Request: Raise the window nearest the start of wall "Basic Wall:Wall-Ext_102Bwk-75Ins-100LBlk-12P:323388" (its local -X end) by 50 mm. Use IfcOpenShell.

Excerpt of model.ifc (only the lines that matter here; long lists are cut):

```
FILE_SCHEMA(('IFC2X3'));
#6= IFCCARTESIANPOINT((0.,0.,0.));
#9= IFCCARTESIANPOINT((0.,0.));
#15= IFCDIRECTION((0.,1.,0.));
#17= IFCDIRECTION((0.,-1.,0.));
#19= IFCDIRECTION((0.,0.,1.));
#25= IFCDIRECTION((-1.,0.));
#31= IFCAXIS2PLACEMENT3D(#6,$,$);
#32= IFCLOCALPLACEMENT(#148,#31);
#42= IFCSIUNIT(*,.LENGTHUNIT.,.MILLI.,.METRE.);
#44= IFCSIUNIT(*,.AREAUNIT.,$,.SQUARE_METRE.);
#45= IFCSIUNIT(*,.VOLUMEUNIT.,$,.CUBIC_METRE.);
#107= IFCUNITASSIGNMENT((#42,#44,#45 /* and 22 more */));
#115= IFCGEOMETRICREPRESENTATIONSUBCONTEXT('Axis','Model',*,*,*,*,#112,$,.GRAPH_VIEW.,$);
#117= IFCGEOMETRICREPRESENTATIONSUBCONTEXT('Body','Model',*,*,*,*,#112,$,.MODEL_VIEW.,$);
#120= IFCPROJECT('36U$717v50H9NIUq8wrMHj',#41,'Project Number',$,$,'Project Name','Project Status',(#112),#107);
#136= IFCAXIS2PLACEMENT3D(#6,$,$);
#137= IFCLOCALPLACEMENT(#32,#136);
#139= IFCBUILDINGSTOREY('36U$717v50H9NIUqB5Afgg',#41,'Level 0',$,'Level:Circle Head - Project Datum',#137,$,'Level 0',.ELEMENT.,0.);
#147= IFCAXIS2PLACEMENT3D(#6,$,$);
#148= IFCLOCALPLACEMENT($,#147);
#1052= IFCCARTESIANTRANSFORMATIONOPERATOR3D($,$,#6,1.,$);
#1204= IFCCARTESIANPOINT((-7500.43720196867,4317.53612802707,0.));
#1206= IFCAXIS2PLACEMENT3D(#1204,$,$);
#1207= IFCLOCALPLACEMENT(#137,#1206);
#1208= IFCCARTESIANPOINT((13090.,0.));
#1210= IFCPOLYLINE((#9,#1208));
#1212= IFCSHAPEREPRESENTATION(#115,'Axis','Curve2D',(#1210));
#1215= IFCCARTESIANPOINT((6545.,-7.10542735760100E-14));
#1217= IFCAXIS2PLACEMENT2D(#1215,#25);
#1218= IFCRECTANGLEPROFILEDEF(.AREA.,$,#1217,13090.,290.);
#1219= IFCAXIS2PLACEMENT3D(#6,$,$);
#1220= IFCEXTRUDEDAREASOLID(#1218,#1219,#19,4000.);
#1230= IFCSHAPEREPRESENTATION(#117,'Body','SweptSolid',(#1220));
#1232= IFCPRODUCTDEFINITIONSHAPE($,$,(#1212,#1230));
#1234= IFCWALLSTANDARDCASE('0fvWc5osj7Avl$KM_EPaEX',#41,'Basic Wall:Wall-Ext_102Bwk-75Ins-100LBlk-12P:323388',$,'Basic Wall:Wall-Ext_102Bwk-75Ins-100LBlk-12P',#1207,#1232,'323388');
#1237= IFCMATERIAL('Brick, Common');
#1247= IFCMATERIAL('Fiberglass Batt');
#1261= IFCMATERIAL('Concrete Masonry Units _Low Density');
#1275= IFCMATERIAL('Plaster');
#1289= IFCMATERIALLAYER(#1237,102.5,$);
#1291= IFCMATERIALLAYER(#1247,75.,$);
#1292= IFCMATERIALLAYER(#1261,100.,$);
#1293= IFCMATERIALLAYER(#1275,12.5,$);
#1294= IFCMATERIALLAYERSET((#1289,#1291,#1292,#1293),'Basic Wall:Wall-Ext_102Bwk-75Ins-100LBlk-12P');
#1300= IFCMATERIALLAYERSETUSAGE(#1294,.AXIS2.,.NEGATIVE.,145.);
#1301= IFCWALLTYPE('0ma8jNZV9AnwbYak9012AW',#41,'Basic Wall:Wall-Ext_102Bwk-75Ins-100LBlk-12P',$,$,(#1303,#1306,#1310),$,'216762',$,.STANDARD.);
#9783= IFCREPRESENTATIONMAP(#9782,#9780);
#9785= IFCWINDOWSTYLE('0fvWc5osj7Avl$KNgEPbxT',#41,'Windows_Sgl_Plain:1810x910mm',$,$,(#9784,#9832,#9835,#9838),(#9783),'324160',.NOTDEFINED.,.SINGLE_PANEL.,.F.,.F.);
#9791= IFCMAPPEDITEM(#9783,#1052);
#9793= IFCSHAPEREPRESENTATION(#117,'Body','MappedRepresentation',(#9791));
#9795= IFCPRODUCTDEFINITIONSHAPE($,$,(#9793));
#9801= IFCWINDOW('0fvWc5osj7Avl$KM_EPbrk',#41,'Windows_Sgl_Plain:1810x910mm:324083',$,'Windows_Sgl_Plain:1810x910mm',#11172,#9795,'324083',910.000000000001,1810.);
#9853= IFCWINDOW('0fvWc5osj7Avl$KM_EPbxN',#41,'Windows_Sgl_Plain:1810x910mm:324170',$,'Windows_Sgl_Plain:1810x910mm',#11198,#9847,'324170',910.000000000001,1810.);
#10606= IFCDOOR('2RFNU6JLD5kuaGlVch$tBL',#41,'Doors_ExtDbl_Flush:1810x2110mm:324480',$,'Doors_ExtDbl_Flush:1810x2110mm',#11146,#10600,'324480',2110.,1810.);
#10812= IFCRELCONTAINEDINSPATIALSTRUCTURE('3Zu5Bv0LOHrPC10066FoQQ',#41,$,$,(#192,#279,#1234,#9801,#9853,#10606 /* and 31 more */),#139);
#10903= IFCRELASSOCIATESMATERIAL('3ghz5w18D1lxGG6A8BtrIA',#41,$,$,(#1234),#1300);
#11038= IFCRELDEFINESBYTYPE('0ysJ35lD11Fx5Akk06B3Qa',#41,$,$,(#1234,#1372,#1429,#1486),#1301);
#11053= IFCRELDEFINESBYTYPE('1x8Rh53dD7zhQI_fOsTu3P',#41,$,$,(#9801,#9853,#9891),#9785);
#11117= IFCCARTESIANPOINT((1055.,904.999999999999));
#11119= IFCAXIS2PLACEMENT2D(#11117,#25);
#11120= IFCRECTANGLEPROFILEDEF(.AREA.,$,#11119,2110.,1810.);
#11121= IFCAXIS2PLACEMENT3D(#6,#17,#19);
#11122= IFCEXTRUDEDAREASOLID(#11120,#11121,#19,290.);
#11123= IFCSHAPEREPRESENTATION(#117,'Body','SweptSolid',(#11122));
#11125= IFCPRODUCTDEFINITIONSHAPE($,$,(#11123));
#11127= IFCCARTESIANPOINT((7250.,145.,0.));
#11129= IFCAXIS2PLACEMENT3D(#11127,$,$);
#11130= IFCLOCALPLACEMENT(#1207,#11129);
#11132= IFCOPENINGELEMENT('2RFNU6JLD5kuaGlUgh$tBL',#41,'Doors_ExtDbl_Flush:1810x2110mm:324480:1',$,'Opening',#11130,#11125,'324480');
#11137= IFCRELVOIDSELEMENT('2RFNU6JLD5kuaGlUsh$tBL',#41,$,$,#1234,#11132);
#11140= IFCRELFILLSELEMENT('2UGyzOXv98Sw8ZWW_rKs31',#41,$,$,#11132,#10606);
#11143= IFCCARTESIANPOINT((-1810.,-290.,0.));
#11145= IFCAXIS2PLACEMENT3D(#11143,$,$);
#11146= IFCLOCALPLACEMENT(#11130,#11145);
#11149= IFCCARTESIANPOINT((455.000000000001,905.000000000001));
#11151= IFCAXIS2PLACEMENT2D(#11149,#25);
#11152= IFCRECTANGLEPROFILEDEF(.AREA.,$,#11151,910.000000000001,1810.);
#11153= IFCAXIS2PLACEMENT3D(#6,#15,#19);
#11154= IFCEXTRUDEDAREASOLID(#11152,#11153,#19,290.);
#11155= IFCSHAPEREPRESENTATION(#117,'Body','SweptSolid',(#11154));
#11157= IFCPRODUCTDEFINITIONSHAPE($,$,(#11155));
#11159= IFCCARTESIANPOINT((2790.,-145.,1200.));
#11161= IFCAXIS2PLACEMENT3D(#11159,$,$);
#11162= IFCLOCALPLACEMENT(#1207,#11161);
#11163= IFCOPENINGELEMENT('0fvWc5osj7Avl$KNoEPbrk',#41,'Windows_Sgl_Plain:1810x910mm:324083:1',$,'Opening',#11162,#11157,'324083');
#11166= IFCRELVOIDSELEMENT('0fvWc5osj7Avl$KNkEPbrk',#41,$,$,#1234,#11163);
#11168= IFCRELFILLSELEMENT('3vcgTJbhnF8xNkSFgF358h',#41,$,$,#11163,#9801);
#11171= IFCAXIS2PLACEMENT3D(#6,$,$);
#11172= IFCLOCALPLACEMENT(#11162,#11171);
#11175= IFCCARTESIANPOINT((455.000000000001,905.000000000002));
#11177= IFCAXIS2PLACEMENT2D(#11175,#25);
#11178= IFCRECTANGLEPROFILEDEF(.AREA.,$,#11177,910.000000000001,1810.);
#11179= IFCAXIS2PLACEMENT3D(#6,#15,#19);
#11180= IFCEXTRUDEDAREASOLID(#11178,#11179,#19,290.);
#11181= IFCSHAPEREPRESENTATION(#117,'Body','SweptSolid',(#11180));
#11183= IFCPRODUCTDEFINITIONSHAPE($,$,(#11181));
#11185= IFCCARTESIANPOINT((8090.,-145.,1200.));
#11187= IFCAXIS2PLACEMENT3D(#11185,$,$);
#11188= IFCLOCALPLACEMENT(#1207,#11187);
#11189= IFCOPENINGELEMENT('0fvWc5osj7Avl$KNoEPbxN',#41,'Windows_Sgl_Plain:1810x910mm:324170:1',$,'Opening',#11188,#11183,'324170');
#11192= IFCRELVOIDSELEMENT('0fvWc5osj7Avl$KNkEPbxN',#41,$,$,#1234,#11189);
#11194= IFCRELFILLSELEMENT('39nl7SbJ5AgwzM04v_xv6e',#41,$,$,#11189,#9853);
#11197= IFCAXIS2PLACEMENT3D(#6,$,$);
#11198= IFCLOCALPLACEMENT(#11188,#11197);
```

```python
import numpy as np
import ifcopenshell
import ifcopenshell.api.geometry
import ifcopenshell.util.placement
import ifcopenshell.util.unit

model = ifcopenshell.open("model.ifc")
unit_scale = ifcopenshell.util.unit.calculate_unit_scale(model)

window = model.by_guid("0fvWc5osj7Avl$KM_EPbrk")
opening = window.FillsVoids[0].RelatingOpeningElement
dz = 0.05 / unit_scale

shift = np.array([0.0, 0.0, dz])
# The window is placed relative to its opening, so it follows when the opening moves.
matrix = ifcopenshell.util.placement.get_local_placement(opening.ObjectPlacement)
matrix[:3, 3] += shift
ifcopenshell.api.geometry.edit_object_placement(
    model, product=opening, matrix=matrix, is_si=False, should_transform_children=True
)

print(f"moved by {dz * unit_scale:+.3f} m")

model.write("model-out.ifc")
```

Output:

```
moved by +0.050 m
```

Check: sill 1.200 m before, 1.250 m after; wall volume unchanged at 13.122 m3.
